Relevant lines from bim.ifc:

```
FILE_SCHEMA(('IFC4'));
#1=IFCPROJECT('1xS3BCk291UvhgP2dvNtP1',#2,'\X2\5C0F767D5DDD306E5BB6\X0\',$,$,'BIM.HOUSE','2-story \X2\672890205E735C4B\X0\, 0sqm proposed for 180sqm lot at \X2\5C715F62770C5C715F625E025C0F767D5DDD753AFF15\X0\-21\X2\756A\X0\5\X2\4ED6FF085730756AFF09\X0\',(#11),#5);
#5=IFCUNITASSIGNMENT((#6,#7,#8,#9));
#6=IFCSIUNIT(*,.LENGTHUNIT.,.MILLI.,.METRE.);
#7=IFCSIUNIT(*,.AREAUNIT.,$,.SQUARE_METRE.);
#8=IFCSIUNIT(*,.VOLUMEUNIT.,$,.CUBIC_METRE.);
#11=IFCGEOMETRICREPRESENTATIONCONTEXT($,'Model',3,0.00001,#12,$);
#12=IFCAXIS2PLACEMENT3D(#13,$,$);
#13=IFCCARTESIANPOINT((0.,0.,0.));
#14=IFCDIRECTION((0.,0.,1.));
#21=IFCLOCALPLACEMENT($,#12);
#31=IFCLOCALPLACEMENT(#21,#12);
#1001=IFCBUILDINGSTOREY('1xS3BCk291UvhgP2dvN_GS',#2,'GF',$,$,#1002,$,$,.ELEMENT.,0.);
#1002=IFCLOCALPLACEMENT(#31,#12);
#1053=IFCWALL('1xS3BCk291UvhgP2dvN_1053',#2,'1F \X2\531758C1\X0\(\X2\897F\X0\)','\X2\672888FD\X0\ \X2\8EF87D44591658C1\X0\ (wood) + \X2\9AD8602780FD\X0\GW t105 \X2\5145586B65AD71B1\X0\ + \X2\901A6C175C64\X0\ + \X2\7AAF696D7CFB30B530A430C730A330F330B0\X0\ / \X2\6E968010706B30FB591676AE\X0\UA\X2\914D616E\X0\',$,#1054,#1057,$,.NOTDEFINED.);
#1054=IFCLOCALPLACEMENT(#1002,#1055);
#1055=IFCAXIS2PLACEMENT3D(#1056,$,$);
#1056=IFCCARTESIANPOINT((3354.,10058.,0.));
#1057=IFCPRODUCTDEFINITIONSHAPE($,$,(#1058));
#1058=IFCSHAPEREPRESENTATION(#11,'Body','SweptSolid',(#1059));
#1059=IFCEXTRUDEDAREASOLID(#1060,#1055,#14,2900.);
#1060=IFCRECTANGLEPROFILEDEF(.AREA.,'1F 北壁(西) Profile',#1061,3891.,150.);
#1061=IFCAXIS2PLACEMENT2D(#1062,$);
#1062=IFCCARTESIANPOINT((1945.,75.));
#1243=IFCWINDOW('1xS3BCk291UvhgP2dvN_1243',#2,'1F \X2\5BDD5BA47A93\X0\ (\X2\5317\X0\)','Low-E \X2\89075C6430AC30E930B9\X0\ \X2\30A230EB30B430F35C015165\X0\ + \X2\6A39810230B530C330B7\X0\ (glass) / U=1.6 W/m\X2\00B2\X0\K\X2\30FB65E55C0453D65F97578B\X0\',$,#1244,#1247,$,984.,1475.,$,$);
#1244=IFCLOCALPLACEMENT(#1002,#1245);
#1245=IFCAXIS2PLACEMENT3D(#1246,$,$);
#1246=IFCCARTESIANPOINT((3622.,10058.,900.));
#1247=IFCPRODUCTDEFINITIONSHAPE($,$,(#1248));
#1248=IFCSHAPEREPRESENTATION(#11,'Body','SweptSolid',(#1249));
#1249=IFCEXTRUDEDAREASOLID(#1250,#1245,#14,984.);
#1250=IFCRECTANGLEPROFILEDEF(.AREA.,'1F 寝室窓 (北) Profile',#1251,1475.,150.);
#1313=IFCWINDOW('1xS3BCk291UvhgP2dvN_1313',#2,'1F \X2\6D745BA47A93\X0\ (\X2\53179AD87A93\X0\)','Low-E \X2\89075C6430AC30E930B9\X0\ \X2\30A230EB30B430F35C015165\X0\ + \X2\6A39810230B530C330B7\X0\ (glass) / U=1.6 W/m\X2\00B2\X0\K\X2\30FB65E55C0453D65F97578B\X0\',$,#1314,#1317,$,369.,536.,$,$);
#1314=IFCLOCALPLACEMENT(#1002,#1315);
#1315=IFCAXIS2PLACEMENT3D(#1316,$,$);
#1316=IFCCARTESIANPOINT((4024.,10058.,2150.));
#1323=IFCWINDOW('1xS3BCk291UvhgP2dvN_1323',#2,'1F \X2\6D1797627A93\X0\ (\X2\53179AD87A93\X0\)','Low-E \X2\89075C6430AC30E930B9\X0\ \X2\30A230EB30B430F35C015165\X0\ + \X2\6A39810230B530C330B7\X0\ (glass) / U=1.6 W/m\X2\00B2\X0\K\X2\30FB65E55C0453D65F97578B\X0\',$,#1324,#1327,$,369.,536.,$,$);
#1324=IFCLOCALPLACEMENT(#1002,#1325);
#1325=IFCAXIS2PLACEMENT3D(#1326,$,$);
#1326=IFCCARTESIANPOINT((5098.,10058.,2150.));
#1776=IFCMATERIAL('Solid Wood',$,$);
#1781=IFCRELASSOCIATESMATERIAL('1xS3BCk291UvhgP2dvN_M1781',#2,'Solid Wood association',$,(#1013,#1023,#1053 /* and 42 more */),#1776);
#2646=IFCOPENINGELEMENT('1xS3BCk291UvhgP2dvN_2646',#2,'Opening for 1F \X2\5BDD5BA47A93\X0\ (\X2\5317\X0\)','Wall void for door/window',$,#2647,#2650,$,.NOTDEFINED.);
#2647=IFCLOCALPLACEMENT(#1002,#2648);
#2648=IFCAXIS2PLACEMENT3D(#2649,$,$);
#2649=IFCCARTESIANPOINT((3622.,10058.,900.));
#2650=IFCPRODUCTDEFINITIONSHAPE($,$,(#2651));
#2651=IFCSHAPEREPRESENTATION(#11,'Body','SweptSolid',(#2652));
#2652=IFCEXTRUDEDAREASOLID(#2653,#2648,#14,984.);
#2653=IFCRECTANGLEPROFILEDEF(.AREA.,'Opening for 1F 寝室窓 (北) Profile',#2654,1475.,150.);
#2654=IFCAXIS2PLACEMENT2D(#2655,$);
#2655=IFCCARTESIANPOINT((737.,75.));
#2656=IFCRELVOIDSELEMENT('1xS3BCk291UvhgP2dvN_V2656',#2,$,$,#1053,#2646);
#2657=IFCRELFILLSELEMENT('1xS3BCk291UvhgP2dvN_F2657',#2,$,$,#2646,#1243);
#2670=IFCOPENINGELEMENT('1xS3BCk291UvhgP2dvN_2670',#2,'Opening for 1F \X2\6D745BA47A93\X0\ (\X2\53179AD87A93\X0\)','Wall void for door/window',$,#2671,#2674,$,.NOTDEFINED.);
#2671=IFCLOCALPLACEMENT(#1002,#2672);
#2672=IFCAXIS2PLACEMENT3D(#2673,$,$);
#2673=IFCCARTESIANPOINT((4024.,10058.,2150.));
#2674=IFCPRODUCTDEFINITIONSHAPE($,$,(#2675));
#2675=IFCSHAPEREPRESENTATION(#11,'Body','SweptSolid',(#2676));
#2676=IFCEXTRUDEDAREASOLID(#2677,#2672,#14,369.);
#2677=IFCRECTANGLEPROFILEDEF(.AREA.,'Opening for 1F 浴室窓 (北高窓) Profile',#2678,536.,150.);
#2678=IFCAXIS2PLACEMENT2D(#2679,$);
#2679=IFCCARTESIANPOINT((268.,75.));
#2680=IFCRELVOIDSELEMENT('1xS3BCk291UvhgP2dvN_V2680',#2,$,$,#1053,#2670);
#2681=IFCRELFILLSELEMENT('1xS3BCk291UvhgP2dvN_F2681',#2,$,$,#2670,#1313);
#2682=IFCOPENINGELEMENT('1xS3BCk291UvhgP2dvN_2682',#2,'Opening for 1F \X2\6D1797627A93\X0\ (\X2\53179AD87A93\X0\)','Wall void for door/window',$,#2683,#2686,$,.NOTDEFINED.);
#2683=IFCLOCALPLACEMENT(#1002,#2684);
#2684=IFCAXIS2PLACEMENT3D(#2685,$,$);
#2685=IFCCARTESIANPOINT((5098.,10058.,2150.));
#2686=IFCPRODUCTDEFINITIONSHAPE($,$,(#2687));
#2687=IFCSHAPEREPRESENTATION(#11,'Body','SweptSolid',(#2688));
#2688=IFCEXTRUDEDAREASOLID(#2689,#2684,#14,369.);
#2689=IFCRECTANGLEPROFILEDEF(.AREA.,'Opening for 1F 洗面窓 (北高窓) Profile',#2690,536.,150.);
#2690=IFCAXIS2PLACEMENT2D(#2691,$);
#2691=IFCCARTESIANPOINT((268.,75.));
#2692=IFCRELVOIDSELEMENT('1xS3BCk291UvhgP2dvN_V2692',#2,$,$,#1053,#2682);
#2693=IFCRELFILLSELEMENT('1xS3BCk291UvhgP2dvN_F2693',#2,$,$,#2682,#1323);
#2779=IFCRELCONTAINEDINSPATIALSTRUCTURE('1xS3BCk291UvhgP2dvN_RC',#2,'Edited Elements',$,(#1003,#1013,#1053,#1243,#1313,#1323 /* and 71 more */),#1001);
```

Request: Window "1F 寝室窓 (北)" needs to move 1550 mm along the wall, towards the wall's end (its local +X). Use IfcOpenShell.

```python
import ifcopenshell
import ifcopenshell.api.geometry
import ifcopenshell.util.placement

model = ifcopenshell.open("bim.ifc")

window = model.by_id(1243)
opening = window.FillsVoids[0].RelatingOpeningElement
wall = opening.VoidsElements[0].RelatingBuildingElement

wall_matrix = ifcopenshell.util.placement.get_local_placement(wall.ObjectPlacement)
shift = wall_matrix[:3, 0] * 1550.0
before = ifcopenshell.util.placement.get_local_placement(window.ObjectPlacement)[:3, 3].copy()

# The window is not placed relative to its opening, so move both.
for product in (opening, window):
    matrix = ifcopenshell.util.placement.get_local_placement(product.ObjectPlacement)
    matrix[:3, 3] += shift
    ifcopenshell.api.geometry.edit_object_placement(model, product=product, matrix=matrix, is_si=False)

after = ifcopenshell.util.placement.get_local_placement(window.ObjectPlacement)[:3, 3]
print("window moved by", (after - before).round(3) + 0.0)

model.write("bim_edited.ifc")
```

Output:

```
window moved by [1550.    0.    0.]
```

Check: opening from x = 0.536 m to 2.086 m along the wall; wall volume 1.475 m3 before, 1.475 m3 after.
